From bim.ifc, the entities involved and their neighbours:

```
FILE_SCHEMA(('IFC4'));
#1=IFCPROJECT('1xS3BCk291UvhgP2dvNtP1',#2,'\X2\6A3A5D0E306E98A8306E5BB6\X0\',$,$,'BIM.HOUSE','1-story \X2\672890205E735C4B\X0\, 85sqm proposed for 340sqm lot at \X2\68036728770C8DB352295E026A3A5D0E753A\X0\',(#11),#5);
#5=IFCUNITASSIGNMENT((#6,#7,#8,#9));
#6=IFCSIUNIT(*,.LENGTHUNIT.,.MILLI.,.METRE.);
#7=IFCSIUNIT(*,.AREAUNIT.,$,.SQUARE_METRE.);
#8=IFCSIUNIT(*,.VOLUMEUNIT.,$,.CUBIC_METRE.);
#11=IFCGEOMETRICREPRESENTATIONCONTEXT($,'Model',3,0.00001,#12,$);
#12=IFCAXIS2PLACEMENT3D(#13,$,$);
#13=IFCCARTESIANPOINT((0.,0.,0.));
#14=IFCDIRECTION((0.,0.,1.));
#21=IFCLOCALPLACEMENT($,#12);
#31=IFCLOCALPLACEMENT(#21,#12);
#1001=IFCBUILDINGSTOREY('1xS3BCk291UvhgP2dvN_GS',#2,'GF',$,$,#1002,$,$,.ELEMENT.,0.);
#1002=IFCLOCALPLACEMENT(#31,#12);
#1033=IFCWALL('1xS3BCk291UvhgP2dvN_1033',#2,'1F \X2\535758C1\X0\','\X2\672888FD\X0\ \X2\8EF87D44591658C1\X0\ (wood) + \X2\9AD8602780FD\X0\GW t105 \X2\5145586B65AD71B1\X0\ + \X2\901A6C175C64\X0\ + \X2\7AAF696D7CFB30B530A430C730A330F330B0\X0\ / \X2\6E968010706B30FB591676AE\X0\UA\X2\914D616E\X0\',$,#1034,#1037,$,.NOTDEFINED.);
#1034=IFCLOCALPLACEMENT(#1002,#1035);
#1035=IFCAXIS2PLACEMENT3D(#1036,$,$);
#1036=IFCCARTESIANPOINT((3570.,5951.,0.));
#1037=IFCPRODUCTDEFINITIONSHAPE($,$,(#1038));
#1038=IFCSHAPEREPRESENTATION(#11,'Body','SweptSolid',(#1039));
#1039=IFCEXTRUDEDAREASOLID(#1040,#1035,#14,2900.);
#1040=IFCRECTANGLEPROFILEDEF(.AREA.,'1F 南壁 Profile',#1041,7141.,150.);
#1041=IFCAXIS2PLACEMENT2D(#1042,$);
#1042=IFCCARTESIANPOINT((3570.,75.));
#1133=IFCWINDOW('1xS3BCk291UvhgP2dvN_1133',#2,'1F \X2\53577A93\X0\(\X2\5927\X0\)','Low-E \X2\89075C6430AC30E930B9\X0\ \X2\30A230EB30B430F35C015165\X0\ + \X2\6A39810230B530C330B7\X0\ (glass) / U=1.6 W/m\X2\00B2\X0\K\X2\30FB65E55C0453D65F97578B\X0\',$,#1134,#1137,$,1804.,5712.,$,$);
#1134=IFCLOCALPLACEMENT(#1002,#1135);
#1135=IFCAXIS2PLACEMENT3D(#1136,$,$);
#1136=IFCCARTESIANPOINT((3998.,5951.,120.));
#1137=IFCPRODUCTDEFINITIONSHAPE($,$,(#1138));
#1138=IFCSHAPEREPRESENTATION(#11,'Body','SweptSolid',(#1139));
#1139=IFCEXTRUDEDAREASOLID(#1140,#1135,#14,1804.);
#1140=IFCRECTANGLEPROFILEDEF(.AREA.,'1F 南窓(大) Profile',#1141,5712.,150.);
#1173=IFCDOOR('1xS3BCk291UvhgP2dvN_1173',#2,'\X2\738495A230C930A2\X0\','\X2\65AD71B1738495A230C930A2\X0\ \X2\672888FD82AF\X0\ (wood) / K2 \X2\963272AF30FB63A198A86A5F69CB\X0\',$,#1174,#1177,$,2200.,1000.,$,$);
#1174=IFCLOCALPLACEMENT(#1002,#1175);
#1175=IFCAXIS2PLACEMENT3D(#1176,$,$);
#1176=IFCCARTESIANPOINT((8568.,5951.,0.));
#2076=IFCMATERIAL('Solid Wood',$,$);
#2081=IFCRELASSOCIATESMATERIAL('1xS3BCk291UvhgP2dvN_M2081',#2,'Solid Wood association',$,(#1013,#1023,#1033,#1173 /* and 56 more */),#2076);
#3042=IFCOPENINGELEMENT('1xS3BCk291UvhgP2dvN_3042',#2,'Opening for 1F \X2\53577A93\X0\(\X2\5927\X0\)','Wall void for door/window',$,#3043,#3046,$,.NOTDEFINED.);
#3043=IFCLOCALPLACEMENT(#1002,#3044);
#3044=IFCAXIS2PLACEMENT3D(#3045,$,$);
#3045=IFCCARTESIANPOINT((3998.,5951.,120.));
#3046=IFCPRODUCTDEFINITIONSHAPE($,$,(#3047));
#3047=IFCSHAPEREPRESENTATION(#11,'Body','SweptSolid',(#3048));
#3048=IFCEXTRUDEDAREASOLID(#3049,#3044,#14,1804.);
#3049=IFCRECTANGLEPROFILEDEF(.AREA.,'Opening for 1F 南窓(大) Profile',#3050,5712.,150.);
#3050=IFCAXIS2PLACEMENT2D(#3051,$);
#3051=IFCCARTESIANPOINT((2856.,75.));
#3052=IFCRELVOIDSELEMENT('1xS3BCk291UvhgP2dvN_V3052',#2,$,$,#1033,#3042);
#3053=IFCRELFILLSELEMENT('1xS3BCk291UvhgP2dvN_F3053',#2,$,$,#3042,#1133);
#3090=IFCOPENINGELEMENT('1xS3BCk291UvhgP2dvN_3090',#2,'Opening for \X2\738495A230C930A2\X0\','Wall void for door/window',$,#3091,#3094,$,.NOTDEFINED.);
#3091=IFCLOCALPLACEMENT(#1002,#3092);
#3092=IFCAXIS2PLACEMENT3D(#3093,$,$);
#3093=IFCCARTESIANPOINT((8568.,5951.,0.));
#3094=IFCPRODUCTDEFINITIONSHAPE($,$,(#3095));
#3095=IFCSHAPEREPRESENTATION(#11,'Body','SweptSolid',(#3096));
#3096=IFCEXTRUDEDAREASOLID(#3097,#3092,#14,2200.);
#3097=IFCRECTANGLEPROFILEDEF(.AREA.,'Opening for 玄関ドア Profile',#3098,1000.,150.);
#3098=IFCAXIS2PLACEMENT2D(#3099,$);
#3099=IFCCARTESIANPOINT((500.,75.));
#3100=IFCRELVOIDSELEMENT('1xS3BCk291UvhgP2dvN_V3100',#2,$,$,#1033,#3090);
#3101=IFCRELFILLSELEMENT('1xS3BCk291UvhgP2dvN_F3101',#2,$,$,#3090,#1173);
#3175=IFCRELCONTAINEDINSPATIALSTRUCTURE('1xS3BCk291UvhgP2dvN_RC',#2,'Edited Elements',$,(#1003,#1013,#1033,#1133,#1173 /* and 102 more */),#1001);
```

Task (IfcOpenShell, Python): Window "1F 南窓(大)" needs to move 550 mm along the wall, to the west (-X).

```python
import ifcopenshell
import ifcopenshell.api.geometry
import ifcopenshell.util.placement
import ifcopenshell.util.unit

model = ifcopenshell.open("bim.ifc")
unit_scale = ifcopenshell.util.unit.calculate_unit_scale(model)

window = model.by_id(1133)
opening = window.FillsVoids[0].RelatingOpeningElement
wall = opening.VoidsElements[0].RelatingBuildingElement

wall_matrix = ifcopenshell.util.placement.get_local_placement(wall.ObjectPlacement)
shift = wall_matrix[:3, 0] * -0.55 / unit_scale
before = ifcopenshell.util.placement.get_local_placement(window.ObjectPlacement)[:3, 3].copy()

# The window is not placed relative to its opening, so move both.
for product in (opening, window):
    matrix = ifcopenshell.util.placement.get_local_placement(product.ObjectPlacement)
    matrix[:3, 3] += shift
    ifcopenshell.api.geometry.edit_object_placement(model, product=product, matrix=matrix, is_si=False)

after = ifcopenshell.util.placement.get_local_placement(window.ObjectPlacement)[:3, 3]
print("window moved by", (after - before).round(3) + 0.0)

model.write("bim_v2.ifc")
```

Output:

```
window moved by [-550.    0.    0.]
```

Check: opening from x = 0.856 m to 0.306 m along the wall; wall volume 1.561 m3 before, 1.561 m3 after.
